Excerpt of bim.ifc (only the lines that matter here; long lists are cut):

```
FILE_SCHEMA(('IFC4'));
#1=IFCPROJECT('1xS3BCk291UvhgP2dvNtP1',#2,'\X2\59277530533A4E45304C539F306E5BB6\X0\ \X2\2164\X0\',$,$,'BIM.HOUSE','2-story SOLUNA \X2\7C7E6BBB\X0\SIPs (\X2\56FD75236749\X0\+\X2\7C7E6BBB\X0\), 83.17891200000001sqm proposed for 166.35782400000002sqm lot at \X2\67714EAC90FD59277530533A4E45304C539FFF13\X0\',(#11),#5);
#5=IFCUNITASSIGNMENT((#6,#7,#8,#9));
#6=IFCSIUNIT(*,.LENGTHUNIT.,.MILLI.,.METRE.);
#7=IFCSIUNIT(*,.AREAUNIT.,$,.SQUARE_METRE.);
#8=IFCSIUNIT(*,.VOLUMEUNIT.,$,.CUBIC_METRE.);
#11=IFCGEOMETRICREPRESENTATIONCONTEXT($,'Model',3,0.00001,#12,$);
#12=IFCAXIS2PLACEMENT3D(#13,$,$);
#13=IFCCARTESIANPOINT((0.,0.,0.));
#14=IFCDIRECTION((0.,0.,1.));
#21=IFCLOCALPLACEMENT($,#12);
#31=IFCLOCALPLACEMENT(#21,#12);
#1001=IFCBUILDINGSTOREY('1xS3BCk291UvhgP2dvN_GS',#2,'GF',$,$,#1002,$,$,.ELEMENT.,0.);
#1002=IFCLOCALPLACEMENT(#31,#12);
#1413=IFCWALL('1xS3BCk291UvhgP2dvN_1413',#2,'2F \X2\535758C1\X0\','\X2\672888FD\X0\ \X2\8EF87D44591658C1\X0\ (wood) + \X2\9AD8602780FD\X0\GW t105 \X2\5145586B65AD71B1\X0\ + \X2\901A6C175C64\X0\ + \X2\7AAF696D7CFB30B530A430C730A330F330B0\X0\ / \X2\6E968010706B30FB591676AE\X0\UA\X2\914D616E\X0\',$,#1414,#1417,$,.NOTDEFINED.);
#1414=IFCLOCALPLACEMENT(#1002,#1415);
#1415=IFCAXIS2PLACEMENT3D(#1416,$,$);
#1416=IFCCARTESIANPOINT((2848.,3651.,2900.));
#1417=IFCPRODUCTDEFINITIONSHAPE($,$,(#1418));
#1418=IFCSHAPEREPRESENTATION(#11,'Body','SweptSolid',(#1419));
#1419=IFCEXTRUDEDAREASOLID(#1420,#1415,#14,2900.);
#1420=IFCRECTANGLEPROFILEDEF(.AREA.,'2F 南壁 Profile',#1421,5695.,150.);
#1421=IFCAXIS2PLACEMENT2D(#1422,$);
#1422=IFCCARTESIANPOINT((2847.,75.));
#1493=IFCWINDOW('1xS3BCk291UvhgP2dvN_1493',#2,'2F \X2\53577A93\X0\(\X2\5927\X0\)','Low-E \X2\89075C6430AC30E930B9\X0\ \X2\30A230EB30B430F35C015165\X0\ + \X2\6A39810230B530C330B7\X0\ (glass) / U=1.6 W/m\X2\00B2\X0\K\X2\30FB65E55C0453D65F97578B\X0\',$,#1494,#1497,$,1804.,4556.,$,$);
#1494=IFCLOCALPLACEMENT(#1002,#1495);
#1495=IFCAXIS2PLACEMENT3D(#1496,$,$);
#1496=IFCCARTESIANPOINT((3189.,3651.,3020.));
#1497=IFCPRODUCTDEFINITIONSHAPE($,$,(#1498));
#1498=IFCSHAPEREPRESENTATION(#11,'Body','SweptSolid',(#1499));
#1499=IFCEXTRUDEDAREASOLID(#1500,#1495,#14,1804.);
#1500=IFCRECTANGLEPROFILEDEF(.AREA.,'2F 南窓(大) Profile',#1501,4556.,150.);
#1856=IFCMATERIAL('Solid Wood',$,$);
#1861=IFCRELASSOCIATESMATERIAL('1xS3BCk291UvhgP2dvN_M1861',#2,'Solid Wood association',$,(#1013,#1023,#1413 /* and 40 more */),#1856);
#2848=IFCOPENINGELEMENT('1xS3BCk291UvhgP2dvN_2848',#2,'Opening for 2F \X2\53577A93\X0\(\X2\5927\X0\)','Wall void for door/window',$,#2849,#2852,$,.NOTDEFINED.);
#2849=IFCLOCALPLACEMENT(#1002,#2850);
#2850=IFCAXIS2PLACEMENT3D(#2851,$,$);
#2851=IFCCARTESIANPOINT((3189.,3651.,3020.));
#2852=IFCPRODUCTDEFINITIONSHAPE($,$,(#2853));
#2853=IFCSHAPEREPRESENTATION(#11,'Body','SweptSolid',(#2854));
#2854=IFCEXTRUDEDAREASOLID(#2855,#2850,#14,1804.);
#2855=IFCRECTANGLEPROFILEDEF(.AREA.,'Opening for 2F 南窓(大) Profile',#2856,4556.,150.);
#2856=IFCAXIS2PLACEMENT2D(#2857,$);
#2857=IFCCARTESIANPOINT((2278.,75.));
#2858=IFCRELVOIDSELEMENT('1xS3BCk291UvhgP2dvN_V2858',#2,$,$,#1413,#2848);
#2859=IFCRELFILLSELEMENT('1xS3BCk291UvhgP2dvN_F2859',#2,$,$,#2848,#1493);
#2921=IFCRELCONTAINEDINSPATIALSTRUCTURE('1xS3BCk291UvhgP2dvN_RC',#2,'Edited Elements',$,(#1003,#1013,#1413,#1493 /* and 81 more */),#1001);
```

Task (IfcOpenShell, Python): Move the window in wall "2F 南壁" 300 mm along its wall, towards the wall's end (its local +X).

```python
import ifcopenshell
import ifcopenshell.api.geometry
import ifcopenshell.util.placement
import ifcopenshell.util.unit

model = ifcopenshell.open("bim.ifc")
unit_scale = ifcopenshell.util.unit.calculate_unit_scale(model)

window = model.by_guid("1xS3BCk291UvhgP2dvN_1493")
opening = window.FillsVoids[0].RelatingOpeningElement
wall = opening.VoidsElements[0].RelatingBuildingElement

wall_matrix = ifcopenshell.util.placement.get_local_placement(wall.ObjectPlacement)
shift = wall_matrix[:3, 0] * 0.3 / unit_scale
before = ifcopenshell.util.placement.get_local_placement(window.ObjectPlacement)[:3, 3].copy()

# The window is not placed relative to its opening, so move both.
for product in (opening, window):
    matrix = ifcopenshell.util.placement.get_local_placement(product.ObjectPlacement)
    matrix[:3, 3] += shift
    ifcopenshell.api.geometry.edit_object_placement(model, product=product, matrix=matrix, is_si=False)

after = ifcopenshell.util.placement.get_local_placement(window.ObjectPlacement)[:3, 3]
print("window moved by", (after - before).round(3) + 0.0)

model.write("bim_updated.ifc")
```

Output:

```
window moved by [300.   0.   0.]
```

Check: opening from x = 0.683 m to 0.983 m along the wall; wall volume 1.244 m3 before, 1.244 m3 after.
